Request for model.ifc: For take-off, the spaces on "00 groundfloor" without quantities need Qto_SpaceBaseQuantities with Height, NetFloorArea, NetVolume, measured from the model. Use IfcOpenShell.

First a look at what the model holds.

```python
import ifcopenshell
import ifcopenshell.util.element
import ifcopenshell.util.unit

model = ifcopenshell.open("model.ifc")
print(model.schema)
for unit_type in ("LENGTHUNIT", "AREAUNIT", "VOLUMEUNIT"):
    print(unit_type, ifcopenshell.util.unit.calculate_unit_scale(model, unit_type))
storey = next(s for s in model.by_type("IfcBuildingStorey") if s.Name == "00 groundfloor")
spaces = [e for e in ifcopenshell.util.element.get_decomposition(storey) if e.is_a("IfcSpace")]
for e in sorted(spaces, key=lambda e: e.id()):
    print(e.id(), e.is_a(), e.Name, list(ifcopenshell.util.element.get_psets(e, qtos_only=True)), sep=" | ")
```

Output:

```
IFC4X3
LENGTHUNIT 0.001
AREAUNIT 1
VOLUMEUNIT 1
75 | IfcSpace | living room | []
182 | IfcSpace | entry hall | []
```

```python
import ifcopenshell
import ifcopenshell.api.pset
import ifcopenshell.geom
import ifcopenshell.util.element
import ifcopenshell.util.shape
import ifcopenshell.util.unit

model = ifcopenshell.open("model.ifc")
unit_scale = ifcopenshell.util.unit.calculate_unit_scale(model)
area_scale = ifcopenshell.util.unit.calculate_unit_scale(model, "AREAUNIT")
volume_scale = ifcopenshell.util.unit.calculate_unit_scale(model, "VOLUMEUNIT")
settings = ifcopenshell.geom.settings()

storey = next(s for s in model.by_type("IfcBuildingStorey") if s.Name == "00 groundfloor")
spaces = [e for e in ifcopenshell.util.element.get_decomposition(storey) if e.is_a("IfcSpace")]

for e in sorted(spaces, key=lambda e: e.id()):
    if ifcopenshell.util.element.get_psets(e, qtos_only=True, should_inherit=False):
        continue
    # Geometry comes back in metres, in the element's own axes.
    shape = ifcopenshell.geom.create_shape(settings, e)
    values = {
        "Height": ifcopenshell.util.shape.get_z(shape.geometry) / unit_scale,
        "NetFloorArea": ifcopenshell.util.shape.get_footprint_area(shape.geometry) / area_scale,
        "NetVolume": ifcopenshell.util.shape.get_volume(shape.geometry) / volume_scale,
    }
    qto = ifcopenshell.api.pset.add_qto(model, product=e, name="Qto_SpaceBaseQuantities")
    ifcopenshell.api.pset.edit_qto(model, qto=qto, properties=values)
    print(e.id(), {k: round(v, 3) for k, v in values.items()})

model.write("model-out.ifc")
```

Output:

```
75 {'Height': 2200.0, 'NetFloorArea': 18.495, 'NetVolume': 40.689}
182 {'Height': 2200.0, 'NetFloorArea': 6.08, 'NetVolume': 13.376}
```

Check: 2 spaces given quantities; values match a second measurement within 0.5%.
